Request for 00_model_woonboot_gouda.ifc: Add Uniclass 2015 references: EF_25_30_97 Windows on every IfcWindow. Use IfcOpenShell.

First a look at what the model holds.

```python
import ifcopenshell

model = ifcopenshell.open("00_model_woonboot_gouda.ifc")
print(model.schema)
print("classifications:", [c.Name for c in model.by_type("IfcClassification")])
for ifc_class in ("IfcDoor", "IfcRoof", "IfcStair", "IfcWall", "IfcWindow"):
    print(ifc_class, len(model.by_type(ifc_class)))
```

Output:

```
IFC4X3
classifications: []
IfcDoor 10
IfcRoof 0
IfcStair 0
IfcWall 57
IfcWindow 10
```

```python
import ifcopenshell
import ifcopenshell.api.classification

model = ifcopenshell.open("00_model_woonboot_gouda.ifc")

system = ifcopenshell.api.classification.add_classification(model, classification="Uniclass 2015")

codes = {
    "IfcWindow": ("EF_25_30_97", "Windows"),
}
for ifc_class, (code, name) in codes.items():
    products = model.by_type(ifc_class)
    ifcopenshell.api.classification.add_reference(
        model, products=products, classification=system, identification=code, name=name
    )
    print(code, len(products))

model.write("00_model_woonboot_gouda_edited.ifc")
```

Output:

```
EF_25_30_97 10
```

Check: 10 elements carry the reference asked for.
